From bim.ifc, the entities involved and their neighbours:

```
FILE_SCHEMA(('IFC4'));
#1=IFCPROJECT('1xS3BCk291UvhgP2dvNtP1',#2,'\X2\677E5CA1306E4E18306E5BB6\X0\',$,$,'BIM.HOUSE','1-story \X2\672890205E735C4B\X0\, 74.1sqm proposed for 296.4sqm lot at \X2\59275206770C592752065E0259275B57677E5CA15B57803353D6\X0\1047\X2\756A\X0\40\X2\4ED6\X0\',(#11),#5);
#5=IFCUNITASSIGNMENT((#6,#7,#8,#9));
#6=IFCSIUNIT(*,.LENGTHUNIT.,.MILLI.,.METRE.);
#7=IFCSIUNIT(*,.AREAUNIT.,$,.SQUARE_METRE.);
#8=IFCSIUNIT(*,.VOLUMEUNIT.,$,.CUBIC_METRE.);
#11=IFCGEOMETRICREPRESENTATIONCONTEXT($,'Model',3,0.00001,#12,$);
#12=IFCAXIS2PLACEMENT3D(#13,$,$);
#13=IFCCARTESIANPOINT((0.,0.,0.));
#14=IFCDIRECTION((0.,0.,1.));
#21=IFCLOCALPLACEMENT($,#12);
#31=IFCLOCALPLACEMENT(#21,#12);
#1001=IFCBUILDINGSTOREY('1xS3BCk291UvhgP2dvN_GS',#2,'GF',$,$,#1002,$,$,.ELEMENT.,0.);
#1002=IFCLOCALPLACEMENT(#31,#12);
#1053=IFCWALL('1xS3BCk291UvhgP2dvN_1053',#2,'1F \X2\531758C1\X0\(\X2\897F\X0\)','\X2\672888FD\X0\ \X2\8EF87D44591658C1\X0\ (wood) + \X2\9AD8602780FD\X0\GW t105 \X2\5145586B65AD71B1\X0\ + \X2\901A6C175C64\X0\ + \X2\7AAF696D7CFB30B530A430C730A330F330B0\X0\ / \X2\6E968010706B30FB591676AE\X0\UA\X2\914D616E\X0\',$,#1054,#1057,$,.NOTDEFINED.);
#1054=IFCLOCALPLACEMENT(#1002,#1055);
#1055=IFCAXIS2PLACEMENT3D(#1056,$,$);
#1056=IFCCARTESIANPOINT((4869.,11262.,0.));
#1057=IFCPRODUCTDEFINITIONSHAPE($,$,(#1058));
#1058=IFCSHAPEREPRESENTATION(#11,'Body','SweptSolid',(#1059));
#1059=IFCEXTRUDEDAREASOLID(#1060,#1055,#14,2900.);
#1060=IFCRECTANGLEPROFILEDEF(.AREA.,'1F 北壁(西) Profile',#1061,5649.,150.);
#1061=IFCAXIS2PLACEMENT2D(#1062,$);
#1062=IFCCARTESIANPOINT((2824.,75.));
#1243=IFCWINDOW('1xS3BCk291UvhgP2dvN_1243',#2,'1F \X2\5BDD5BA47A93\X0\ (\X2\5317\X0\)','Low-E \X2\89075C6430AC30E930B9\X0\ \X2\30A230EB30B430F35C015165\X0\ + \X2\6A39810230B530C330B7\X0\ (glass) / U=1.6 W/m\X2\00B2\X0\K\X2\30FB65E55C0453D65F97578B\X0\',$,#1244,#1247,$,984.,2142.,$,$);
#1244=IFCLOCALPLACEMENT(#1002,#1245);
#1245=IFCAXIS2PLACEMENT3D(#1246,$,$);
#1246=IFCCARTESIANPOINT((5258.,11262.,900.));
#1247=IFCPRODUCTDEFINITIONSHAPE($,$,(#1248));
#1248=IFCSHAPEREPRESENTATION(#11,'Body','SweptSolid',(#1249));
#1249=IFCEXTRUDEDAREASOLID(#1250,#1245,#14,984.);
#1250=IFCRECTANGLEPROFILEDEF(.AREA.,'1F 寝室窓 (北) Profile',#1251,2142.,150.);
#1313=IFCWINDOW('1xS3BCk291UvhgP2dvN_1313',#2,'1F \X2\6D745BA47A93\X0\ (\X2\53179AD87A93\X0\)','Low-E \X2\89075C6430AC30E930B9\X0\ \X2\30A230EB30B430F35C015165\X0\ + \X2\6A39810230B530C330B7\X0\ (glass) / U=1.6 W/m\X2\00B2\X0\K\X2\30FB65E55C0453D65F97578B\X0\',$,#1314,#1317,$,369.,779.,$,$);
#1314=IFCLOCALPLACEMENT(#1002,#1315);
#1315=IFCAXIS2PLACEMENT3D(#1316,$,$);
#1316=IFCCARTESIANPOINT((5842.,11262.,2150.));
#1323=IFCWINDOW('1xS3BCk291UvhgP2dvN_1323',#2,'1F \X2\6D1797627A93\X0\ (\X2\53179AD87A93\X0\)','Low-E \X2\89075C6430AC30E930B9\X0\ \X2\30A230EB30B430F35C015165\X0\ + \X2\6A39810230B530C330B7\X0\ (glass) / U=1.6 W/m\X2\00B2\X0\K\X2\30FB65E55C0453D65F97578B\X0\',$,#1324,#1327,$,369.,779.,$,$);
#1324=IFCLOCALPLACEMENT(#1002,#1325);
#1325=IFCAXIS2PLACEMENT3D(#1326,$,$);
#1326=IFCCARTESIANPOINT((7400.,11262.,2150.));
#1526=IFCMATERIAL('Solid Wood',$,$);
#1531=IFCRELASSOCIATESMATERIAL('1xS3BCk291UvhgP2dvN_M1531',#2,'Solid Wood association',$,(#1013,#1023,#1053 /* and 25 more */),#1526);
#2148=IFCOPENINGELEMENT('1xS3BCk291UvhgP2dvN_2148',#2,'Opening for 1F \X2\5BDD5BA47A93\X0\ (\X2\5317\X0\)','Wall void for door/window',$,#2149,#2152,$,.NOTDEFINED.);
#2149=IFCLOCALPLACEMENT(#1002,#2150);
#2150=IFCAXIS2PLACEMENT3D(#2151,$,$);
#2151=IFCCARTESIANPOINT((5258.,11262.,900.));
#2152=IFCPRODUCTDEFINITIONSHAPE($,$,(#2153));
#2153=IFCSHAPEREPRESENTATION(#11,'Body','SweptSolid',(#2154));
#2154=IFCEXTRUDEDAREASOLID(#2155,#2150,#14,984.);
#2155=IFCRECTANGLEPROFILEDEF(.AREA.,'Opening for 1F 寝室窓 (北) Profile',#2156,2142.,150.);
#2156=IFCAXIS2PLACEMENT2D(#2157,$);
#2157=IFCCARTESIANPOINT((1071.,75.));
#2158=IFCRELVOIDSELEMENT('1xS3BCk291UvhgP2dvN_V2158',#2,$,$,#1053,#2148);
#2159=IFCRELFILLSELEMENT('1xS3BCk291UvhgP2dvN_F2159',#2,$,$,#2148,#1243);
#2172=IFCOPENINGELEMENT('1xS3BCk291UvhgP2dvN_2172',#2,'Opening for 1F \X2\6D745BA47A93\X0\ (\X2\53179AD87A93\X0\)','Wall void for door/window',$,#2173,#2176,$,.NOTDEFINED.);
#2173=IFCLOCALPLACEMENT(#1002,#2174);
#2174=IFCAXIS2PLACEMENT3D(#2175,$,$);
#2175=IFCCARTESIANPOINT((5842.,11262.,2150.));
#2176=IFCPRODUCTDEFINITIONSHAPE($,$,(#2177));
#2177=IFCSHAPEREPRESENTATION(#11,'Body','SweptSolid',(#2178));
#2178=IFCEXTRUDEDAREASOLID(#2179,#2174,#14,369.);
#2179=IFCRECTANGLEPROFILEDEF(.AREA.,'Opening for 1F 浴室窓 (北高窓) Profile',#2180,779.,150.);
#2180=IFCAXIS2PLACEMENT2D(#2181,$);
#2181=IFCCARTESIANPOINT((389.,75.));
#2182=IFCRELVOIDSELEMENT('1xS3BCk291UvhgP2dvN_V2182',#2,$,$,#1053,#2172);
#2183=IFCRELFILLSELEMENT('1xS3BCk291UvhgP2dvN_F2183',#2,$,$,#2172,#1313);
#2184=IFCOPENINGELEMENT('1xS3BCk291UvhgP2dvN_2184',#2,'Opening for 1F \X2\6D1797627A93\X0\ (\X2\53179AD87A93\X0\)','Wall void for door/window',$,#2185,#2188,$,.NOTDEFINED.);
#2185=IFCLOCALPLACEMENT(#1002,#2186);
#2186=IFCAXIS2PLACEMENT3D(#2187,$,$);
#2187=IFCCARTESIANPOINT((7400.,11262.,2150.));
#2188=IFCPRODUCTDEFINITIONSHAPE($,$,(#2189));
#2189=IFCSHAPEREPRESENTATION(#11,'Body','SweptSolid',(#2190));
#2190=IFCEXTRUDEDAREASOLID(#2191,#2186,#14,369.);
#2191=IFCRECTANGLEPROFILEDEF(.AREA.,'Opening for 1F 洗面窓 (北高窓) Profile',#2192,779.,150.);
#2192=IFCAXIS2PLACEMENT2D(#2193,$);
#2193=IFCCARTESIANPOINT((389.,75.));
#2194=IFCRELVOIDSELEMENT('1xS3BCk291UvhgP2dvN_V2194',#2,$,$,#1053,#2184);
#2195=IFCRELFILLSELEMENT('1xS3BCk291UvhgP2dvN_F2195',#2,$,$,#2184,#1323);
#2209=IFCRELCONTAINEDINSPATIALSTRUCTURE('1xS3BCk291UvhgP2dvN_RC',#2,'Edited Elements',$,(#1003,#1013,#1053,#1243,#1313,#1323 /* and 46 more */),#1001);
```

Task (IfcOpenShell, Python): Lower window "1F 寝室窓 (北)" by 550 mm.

```python
import numpy as np
import ifcopenshell
import ifcopenshell.api.geometry
import ifcopenshell.util.placement
import ifcopenshell.util.unit

model = ifcopenshell.open("bim.ifc")
unit_scale = ifcopenshell.util.unit.calculate_unit_scale(model)

window = model.by_id(1243)
opening = window.FillsVoids[0].RelatingOpeningElement
dz = -550.0

shift = np.array([0.0, 0.0, dz])
# The window is not placed relative to its opening, so move both.
for product in (opening, window):
    matrix = ifcopenshell.util.placement.get_local_placement(product.ObjectPlacement)
    matrix[:3, 3] += shift
    ifcopenshell.api.geometry.edit_object_placement(model, product=product, matrix=matrix, is_si=False)

print(f"moved by {dz * unit_scale:+.3f} m")

model.write("bim_edited.ifc")
```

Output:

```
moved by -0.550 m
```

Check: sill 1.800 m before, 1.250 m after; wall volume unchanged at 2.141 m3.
